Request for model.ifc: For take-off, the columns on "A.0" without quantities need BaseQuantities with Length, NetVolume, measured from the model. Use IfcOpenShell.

First a look at what the model holds.

```python
import ifcopenshell
import ifcopenshell.util.element
import ifcopenshell.util.unit

model = ifcopenshell.open("model.ifc")
print(model.schema)
for unit_type in ("LENGTHUNIT", "AREAUNIT", "VOLUMEUNIT"):
    print(unit_type, ifcopenshell.util.unit.calculate_unit_scale(model, unit_type))
storey = next(s for s in model.by_type("IfcBuildingStorey") if s.Name == "A.0")
columns = [e for e in ifcopenshell.util.element.get_decomposition(storey) if e.is_a("IfcColumn")]
for e in sorted(columns, key=lambda e: e.id()):
    print(e.id(), e.is_a(), e.Name, list(ifcopenshell.util.element.get_psets(e, qtos_only=True)), sep=" | ")
```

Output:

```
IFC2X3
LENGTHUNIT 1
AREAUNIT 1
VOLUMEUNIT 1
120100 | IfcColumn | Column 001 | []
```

```python
import ifcopenshell
import ifcopenshell.api.pset
import ifcopenshell.geom
import ifcopenshell.util.element
import ifcopenshell.util.shape
import ifcopenshell.util.unit

model = ifcopenshell.open("model.ifc")
unit_scale = ifcopenshell.util.unit.calculate_unit_scale(model)
volume_scale = ifcopenshell.util.unit.calculate_unit_scale(model, "VOLUMEUNIT")
settings = ifcopenshell.geom.settings()

storey = next(s for s in model.by_type("IfcBuildingStorey") if s.Name == "A.0")
columns = [e for e in ifcopenshell.util.element.get_decomposition(storey) if e.is_a("IfcColumn")]

for e in sorted(columns, key=lambda e: e.id()):
    if ifcopenshell.util.element.get_psets(e, qtos_only=True, should_inherit=False):
        continue
    # Geometry comes back in metres, in the element's own axes.
    shape = ifcopenshell.geom.create_shape(settings, e)
    values = {
        "Length": ifcopenshell.util.shape.get_z(shape.geometry) / unit_scale,
        "NetVolume": ifcopenshell.util.shape.get_volume(shape.geometry) / volume_scale,
    }
    qto = ifcopenshell.api.pset.add_qto(model, product=e, name="BaseQuantities")
    ifcopenshell.api.pset.edit_qto(model, qto=qto, properties=values)
    print(e.id(), {k: round(v, 3) for k, v in values.items()})

model.write("model_v2.ifc")
```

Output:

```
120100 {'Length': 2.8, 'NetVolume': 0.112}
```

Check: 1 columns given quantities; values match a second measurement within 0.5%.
